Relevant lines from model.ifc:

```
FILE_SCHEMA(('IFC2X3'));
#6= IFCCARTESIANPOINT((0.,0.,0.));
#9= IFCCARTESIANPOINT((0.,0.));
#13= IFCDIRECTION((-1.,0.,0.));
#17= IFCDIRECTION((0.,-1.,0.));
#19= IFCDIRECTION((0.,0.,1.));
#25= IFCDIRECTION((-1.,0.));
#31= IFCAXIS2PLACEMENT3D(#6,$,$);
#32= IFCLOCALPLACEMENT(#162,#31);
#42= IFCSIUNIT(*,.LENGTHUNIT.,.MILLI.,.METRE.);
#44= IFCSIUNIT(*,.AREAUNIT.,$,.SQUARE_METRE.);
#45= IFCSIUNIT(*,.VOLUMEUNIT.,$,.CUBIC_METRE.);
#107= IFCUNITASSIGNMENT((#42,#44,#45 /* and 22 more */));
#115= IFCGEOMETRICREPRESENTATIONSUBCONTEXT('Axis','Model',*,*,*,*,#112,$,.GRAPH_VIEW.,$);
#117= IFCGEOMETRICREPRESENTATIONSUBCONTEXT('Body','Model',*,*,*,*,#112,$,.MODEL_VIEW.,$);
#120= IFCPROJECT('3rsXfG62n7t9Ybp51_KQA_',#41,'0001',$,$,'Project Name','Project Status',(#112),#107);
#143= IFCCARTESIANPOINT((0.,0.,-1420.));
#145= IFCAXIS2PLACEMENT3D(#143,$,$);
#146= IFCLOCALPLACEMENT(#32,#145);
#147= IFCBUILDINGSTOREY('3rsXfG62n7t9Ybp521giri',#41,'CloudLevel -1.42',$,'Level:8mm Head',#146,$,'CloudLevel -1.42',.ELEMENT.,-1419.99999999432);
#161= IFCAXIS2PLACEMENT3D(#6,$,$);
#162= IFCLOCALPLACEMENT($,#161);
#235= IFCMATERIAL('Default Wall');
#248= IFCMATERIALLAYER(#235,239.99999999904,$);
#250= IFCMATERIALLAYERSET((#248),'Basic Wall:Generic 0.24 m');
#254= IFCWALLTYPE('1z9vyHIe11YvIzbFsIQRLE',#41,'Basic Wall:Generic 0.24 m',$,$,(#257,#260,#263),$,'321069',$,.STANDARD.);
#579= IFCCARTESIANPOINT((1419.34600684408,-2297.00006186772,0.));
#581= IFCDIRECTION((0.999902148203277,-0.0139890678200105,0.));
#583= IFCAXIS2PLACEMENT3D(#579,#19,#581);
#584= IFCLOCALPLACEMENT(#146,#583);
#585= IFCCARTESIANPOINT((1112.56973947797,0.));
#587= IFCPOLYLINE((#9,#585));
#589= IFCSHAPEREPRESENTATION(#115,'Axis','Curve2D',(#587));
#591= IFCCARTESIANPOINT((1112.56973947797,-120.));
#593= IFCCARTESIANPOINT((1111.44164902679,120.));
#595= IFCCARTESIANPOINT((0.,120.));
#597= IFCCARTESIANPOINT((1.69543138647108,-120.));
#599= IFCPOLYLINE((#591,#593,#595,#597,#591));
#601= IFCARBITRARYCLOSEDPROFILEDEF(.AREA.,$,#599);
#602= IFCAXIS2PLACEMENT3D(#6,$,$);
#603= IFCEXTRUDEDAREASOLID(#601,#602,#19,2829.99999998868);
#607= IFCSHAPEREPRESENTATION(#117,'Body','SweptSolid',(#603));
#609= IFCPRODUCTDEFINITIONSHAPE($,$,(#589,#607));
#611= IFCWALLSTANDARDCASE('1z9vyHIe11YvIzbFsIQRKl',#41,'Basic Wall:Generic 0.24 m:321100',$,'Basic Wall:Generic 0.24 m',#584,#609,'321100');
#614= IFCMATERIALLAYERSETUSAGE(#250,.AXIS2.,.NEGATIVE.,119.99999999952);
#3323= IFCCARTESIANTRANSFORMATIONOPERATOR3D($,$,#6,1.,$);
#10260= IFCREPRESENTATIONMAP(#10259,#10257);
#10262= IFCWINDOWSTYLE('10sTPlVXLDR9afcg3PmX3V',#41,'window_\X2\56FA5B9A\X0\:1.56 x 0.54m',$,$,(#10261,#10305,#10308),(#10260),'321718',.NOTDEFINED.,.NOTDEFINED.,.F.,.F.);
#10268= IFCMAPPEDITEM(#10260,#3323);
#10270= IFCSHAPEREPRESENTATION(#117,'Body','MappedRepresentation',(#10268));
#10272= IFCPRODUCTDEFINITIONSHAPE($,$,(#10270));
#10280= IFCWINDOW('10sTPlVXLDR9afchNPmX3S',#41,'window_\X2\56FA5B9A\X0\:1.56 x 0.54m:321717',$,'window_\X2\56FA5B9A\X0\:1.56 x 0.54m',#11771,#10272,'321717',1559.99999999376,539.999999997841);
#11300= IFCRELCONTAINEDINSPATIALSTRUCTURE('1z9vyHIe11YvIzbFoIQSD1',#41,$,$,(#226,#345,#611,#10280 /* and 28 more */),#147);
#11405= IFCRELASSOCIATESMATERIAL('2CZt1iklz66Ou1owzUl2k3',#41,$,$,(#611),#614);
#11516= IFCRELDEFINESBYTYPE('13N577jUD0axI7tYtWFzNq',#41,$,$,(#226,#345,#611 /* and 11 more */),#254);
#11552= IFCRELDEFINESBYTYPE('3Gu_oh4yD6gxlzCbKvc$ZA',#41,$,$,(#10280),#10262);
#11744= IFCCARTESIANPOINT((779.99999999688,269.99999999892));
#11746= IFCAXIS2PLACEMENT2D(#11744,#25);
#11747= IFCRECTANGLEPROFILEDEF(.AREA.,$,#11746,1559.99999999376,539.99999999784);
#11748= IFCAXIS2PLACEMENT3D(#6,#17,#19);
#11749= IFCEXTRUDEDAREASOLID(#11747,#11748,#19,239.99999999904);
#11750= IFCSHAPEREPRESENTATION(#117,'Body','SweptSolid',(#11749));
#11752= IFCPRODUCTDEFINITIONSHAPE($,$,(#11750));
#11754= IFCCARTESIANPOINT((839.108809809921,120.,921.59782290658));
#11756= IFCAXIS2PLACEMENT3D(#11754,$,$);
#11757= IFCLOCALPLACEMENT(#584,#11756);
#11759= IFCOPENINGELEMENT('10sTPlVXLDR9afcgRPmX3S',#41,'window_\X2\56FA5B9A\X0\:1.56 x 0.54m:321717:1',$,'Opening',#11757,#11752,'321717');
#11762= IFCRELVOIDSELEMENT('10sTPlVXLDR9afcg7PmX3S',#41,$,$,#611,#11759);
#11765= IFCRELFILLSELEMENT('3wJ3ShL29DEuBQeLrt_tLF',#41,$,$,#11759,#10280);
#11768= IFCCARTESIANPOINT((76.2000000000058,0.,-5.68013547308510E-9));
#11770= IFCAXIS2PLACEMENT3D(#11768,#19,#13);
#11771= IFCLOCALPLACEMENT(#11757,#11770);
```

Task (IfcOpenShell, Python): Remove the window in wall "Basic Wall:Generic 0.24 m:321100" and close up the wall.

```python
import ifcopenshell
import ifcopenshell.api.feature
import ifcopenshell.api.root
import ifcopenshell.geom
import ifcopenshell.util.shape

model = ifcopenshell.open("model.ifc")
settings = ifcopenshell.geom.settings()


def volume(element):
    """Net volume in cubic metres, openings subtracted."""
    shape = ifcopenshell.geom.create_shape(settings, element)
    return ifcopenshell.util.shape.get_volume(shape.geometry)


window = model.by_id(10280)
opening = window.FillsVoids[0].RelatingOpeningElement
wall = opening.VoidsElements[0].RelatingBuildingElement
before = volume(wall)

ifcopenshell.api.root.remove_product(model, product=window)
ifcopenshell.api.feature.remove_feature(model, feature=opening)

after = volume(wall)

print(f"wall volume {before:.3f} -> {after:.3f} m3")

model.write("model_rev.ifc")
```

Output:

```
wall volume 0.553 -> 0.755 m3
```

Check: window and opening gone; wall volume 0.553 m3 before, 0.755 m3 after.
